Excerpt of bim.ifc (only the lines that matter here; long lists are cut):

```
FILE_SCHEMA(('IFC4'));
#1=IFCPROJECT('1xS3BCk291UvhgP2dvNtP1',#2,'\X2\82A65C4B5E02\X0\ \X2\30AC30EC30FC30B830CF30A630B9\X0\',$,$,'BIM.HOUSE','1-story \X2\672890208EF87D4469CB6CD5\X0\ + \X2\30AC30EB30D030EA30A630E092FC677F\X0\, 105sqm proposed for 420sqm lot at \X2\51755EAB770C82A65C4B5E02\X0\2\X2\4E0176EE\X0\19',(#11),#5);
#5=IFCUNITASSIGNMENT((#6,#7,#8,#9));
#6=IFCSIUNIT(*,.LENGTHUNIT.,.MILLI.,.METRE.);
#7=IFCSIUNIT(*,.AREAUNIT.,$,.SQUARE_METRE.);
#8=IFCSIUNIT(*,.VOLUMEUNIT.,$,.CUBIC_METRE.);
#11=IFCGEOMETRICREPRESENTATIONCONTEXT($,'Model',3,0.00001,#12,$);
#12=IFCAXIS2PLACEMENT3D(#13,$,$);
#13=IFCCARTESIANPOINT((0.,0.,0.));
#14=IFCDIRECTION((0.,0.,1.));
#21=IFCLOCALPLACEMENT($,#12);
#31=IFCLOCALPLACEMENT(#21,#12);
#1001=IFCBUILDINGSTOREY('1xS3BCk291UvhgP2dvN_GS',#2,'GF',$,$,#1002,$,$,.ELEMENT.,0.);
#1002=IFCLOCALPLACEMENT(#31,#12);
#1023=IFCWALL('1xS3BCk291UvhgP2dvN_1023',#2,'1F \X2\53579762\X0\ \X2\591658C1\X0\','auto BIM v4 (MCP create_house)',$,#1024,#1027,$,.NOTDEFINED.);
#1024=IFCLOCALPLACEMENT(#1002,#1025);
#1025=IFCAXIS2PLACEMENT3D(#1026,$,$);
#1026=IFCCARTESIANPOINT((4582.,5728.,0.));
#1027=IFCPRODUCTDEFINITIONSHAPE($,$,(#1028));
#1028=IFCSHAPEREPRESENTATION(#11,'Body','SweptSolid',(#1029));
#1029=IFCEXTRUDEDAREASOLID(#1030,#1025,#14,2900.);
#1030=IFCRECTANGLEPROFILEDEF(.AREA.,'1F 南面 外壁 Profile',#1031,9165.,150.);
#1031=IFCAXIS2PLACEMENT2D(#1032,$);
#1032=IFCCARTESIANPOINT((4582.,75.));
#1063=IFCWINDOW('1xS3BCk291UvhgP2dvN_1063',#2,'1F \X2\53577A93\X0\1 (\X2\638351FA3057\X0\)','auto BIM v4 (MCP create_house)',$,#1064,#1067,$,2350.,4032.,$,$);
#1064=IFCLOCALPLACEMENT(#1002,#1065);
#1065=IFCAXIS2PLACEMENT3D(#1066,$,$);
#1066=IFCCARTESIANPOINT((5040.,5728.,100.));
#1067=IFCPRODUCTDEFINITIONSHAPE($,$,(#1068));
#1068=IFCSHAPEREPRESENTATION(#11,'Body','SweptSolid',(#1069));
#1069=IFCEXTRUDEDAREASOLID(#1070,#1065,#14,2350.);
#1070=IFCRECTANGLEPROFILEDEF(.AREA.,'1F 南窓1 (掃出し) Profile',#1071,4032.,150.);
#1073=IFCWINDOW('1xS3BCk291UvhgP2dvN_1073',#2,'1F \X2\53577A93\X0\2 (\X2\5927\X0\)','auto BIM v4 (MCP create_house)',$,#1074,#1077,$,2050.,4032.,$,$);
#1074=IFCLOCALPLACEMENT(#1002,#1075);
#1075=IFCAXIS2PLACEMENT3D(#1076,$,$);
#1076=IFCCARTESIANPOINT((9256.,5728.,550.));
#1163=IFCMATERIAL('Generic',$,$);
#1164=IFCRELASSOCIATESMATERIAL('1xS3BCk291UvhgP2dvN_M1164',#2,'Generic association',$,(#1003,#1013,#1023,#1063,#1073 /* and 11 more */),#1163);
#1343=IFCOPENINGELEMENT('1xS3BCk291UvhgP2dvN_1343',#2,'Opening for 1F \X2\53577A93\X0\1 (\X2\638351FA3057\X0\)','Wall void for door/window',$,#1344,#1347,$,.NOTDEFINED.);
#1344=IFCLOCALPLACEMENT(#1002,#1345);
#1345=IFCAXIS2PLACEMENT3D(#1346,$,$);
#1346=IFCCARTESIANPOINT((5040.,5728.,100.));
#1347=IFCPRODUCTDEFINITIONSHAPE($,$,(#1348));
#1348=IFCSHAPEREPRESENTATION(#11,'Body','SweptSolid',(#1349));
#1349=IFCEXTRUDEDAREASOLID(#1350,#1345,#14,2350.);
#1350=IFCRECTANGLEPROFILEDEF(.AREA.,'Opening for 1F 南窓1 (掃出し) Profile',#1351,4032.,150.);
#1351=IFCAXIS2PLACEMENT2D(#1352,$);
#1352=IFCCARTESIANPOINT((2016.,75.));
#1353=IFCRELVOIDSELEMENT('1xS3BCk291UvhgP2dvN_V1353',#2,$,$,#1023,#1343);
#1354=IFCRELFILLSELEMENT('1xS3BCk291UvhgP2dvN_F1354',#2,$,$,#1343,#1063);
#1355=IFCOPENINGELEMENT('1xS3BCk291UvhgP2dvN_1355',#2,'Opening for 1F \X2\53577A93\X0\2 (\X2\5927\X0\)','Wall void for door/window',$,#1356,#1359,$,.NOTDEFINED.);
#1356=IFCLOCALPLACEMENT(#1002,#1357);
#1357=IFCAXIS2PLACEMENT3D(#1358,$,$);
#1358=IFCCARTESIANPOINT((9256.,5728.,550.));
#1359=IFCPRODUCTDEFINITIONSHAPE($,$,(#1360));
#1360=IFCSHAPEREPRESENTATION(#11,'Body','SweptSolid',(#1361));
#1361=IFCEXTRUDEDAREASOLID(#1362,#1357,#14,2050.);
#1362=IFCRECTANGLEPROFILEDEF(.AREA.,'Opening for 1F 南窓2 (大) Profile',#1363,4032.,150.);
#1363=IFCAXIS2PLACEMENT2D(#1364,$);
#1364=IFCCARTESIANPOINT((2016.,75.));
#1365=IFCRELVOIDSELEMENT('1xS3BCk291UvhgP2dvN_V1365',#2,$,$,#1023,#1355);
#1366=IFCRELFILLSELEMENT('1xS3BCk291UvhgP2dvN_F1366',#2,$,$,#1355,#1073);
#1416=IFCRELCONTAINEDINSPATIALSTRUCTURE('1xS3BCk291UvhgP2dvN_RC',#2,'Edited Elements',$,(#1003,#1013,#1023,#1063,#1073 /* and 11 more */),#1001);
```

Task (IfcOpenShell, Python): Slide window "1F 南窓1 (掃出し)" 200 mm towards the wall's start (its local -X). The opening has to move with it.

```python
import ifcopenshell
import ifcopenshell.api.geometry
import ifcopenshell.util.placement
import ifcopenshell.util.unit

model = ifcopenshell.open("bim.ifc")
unit_scale = ifcopenshell.util.unit.calculate_unit_scale(model)

window = model.by_id(1063)
opening = window.FillsVoids[0].RelatingOpeningElement
wall = opening.VoidsElements[0].RelatingBuildingElement

wall_matrix = ifcopenshell.util.placement.get_local_placement(wall.ObjectPlacement)
shift = wall_matrix[:3, 0] * -0.2 / unit_scale
before = ifcopenshell.util.placement.get_local_placement(window.ObjectPlacement)[:3, 3].copy()

# The window is not placed relative to its opening, so move both.
for product in (opening, window):
    matrix = ifcopenshell.util.placement.get_local_placement(product.ObjectPlacement)
    matrix[:3, 3] += shift
    ifcopenshell.api.geometry.edit_object_placement(model, product=product, matrix=matrix, is_si=False)

after = ifcopenshell.util.placement.get_local_placement(window.ObjectPlacement)[:3, 3]
print("window moved by", (after - before).round(3) + 0.0)

model.write("bim-out.ifc")
```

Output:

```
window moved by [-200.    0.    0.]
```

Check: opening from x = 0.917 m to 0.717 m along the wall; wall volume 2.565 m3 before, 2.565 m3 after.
